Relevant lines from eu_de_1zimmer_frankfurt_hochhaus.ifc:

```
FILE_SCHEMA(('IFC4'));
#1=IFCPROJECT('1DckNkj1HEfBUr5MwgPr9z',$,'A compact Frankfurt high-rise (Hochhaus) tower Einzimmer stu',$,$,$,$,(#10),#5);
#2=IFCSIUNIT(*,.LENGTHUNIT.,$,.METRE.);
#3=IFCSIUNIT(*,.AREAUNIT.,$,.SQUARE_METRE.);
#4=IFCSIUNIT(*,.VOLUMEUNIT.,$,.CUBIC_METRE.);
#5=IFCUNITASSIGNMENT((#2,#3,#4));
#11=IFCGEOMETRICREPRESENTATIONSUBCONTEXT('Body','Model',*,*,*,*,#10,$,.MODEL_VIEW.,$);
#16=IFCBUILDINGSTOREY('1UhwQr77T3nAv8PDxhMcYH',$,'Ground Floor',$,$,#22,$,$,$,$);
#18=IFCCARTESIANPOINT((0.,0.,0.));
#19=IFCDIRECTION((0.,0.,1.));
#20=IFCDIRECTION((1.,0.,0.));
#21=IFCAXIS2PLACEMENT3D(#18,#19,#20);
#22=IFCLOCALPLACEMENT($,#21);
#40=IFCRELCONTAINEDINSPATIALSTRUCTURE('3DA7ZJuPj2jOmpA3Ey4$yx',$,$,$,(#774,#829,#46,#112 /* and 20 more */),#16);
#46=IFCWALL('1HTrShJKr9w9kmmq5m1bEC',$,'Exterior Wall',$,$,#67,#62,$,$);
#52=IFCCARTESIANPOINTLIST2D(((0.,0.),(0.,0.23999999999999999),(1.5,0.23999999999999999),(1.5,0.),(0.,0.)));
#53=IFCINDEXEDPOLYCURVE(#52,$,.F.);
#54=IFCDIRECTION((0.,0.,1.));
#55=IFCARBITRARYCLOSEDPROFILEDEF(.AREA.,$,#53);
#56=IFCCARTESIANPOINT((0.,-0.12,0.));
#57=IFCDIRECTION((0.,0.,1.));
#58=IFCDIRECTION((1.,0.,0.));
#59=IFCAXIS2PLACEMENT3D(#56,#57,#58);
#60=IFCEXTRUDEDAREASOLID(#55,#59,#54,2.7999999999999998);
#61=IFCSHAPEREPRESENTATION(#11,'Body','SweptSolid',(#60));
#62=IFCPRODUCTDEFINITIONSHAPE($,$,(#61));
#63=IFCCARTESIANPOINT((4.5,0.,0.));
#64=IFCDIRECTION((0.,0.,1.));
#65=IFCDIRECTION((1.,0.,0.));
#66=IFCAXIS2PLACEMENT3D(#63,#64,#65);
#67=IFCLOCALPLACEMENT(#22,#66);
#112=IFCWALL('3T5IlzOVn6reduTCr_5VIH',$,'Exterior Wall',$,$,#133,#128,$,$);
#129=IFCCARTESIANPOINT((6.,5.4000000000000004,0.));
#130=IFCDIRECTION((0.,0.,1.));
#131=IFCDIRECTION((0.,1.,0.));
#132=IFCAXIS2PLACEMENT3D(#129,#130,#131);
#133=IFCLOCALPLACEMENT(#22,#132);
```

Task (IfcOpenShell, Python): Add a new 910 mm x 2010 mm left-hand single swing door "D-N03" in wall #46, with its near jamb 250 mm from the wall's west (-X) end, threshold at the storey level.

```python
import numpy as np
import ifcopenshell
import ifcopenshell.api.feature
import ifcopenshell.api.geometry
import ifcopenshell.api.root
import ifcopenshell.api.spatial
import ifcopenshell.geom
import ifcopenshell.util.element
import ifcopenshell.util.placement
import ifcopenshell.util.representation
import ifcopenshell.util.shape
import ifcopenshell.util.unit

model = ifcopenshell.open("eu_de_1zimmer_frankfurt_hochhaus.ifc")
unit_scale = ifcopenshell.util.unit.calculate_unit_scale(model)
settings = ifcopenshell.geom.settings()


def volume(element):
    """Net volume in cubic metres, openings subtracted."""
    shape = ifcopenshell.geom.create_shape(settings, element)
    return ifcopenshell.util.shape.get_volume(shape.geometry)


wall = model.by_id(46)
storey = ifcopenshell.util.element.get_container(wall, ifc_class="IfcBuildingStorey")
context = ifcopenshell.util.representation.get_context(model, "Model", "Body", "MODEL_VIEW")
before = volume(wall)

width, height, from_end, sill = 0.91, 2.01, 0.25, 0.0  # metres

# The wall runs along its own X axis, and the end named is its -X end.
wall_shape = ifcopenshell.geom.create_shape(settings, wall)
x, y, z = ifcopenshell.util.shape.get_vertices(wall_shape.geometry).T
start = x.min() + from_end
face, thickness = float(y.min()), float(y.max() - y.min())
wall_matrix = ifcopenshell.util.placement.get_local_placement(wall.ObjectPlacement)
level = ifcopenshell.util.placement.get_local_placement(storey.ObjectPlacement)[2, 3]


def in_wall(x, y):
    """Placement at x, y metres in the wall's axes, at sill height."""
    matrix = wall_matrix.copy()
    matrix[:, 3] = wall_matrix @ np.array([x / unit_scale, y / unit_scale, 0.0, 1.0])
    matrix[2, 3] = level + sill / unit_scale
    return matrix


# Opening: a box that overshoots both wall faces by 50 mm.
opening = ifcopenshell.api.root.create_entity(model, ifc_class="IfcOpeningElement", predefined_type="OPENING")
box = ifcopenshell.api.geometry.add_wall_representation(
    model, context=context, length=width, height=height, thickness=thickness + 0.1
)
ifcopenshell.api.geometry.assign_representation(model, product=opening, representation=box)
ifcopenshell.api.geometry.edit_object_placement(model, product=opening, matrix=in_wall(start, face - 0.05), is_si=False)
ifcopenshell.api.feature.add_feature(model, feature=opening, element=wall)

door = ifcopenshell.api.root.create_entity(model, ifc_class="IfcDoor", name="D-N03", predefined_type="DOOR")
door.OverallWidth, door.OverallHeight = width / unit_scale, height / unit_scale
door.OperationType = "SINGLE_SWING_LEFT"
body = ifcopenshell.api.geometry.add_door_representation(
    model,
    context=context,
    overall_width=door.OverallWidth,
    overall_height=door.OverallHeight,
    operation_type="SINGLE_SWING_LEFT",
    lining_properties={"LiningDepth": thickness / unit_scale, "ThresholdDepth": thickness / unit_scale},
)
ifcopenshell.api.geometry.assign_representation(model, product=door, representation=body)
ifcopenshell.api.spatial.assign_container(model, products=[door], relating_structure=storey)
ifcopenshell.api.feature.add_filling(model, opening=opening, element=door)

# The lining spans the wall, so the door starts at the wall face.
ifcopenshell.api.geometry.edit_object_placement(model, product=door, matrix=in_wall(start, face), is_si=False)

after = volume(wall)

print(f"wall volume {before:.3f} -> {after:.3f} m3")

model.write("eu_de_1zimmer_frankfurt_hochhaus_rev.ifc")
```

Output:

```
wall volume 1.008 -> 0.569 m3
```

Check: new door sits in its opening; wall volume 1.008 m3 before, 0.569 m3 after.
